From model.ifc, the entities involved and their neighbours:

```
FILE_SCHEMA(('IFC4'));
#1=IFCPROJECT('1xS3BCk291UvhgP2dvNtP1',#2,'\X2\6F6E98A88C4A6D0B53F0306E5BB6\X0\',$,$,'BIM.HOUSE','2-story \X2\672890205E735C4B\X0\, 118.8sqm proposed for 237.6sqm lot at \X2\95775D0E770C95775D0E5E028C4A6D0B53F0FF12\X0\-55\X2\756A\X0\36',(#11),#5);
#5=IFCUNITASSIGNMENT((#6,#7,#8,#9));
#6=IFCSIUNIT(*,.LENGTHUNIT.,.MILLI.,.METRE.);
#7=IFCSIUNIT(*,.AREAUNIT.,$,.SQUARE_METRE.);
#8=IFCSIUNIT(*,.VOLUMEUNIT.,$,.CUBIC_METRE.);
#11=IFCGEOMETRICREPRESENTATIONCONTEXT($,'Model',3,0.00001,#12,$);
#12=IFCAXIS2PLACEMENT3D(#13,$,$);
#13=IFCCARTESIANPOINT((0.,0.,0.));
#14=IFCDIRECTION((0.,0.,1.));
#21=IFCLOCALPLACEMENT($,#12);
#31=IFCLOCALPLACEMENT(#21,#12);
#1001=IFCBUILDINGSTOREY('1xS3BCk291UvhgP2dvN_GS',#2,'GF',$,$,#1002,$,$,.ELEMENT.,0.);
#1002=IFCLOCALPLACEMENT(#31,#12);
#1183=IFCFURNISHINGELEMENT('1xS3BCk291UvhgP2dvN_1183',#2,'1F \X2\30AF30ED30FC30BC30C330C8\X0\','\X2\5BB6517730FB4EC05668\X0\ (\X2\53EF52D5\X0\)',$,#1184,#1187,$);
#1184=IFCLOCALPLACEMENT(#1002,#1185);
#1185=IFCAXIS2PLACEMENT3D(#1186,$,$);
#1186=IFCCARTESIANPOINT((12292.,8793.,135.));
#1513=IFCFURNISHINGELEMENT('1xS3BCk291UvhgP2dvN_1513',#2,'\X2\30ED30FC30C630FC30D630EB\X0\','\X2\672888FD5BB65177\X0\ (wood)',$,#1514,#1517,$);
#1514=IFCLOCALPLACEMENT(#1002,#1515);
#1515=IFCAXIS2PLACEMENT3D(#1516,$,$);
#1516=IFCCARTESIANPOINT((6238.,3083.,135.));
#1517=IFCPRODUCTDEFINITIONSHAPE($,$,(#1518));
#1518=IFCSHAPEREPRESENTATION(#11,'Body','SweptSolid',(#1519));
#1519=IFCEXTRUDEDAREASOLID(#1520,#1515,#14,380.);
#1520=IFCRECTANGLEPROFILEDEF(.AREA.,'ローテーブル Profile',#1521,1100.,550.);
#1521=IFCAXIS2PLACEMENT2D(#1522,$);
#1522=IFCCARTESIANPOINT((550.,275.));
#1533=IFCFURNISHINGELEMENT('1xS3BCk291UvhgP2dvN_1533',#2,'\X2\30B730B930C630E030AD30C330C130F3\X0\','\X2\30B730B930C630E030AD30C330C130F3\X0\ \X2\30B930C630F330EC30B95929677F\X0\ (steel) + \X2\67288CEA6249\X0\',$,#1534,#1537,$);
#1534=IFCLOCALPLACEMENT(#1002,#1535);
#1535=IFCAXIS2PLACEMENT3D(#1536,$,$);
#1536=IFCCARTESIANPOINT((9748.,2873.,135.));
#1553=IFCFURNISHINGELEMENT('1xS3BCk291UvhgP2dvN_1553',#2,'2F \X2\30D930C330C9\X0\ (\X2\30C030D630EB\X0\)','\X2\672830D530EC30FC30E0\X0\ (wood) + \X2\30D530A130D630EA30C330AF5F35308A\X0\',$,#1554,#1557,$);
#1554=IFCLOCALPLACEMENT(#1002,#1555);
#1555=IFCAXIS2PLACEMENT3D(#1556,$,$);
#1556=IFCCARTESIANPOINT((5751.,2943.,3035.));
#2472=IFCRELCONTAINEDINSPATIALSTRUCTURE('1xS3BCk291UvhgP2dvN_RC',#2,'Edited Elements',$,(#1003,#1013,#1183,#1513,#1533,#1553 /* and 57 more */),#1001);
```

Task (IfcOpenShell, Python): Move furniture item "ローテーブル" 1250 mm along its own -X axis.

```python
import ifcopenshell
import ifcopenshell.api.geometry
import ifcopenshell.util.placement
import ifcopenshell.util.unit

model = ifcopenshell.open("model.ifc")
unit_scale = ifcopenshell.util.unit.calculate_unit_scale(model)

item = model.by_id(1513)
matrix = ifcopenshell.util.placement.get_local_placement(item.ObjectPlacement)
matrix[:3, 3] -= matrix[:3, 0] * 1.25 / unit_scale
ifcopenshell.api.geometry.edit_object_placement(model, product=item, matrix=matrix, is_si=False)

print(ifcopenshell.util.placement.get_local_placement(item.ObjectPlacement).round(3) + 0.0)

model.write("model_updated.ifc")
```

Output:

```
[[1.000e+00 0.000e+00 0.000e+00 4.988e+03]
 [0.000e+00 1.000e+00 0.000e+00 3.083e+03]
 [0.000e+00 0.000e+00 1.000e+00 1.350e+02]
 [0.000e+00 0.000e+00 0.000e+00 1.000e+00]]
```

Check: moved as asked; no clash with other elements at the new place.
